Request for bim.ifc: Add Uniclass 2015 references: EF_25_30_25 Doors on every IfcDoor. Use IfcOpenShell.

First a look at what the model holds.

```python
import ifcopenshell

model = ifcopenshell.open("bim.ifc")
print(model.schema)
print("classifications:", [c.Name for c in model.by_type("IfcClassification")])
for ifc_class in ("IfcDoor", "IfcRoof", "IfcStair", "IfcWall", "IfcWindow"):
    print(ifc_class, len(model.by_type(ifc_class)))
```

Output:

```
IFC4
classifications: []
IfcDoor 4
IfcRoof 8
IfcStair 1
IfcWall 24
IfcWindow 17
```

```python
import ifcopenshell
import ifcopenshell.api.classification

model = ifcopenshell.open("bim.ifc")

system = ifcopenshell.api.classification.add_classification(model, classification="Uniclass 2015")

codes = {
    "IfcDoor": ("EF_25_30_25", "Doors"),
}
for ifc_class, (code, name) in codes.items():
    products = model.by_type(ifc_class)
    ifcopenshell.api.classification.add_reference(
        model, products=products, classification=system, identification=code, name=name
    )
    print(code, len(products))

model.write("bim-out.ifc")
```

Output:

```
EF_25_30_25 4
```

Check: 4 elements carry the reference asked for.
